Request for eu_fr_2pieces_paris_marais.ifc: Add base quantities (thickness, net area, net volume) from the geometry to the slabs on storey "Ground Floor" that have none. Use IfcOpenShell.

First a look at what the model holds.

```python
import ifcopenshell
import ifcopenshell.util.element
import ifcopenshell.util.unit

model = ifcopenshell.open("eu_fr_2pieces_paris_marais.ifc")
print(model.schema)
for unit_type in ("LENGTHUNIT", "AREAUNIT", "VOLUMEUNIT"):
    print(unit_type, ifcopenshell.util.unit.calculate_unit_scale(model, unit_type))
storey = next(s for s in model.by_type("IfcBuildingStorey") if s.Name == "Ground Floor")
slabs = [e for e in ifcopenshell.util.element.get_decomposition(storey) if e.is_a("IfcSlab")]
for e in sorted(slabs, key=lambda e: e.id()):
    print(e.id(), e.is_a(), e.Name, list(ifcopenshell.util.element.get_psets(e, qtos_only=True)), sep=" | ")
```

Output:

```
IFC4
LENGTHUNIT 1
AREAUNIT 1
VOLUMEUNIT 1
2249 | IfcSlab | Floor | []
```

```python
import ifcopenshell
import ifcopenshell.api.pset
import ifcopenshell.geom
import ifcopenshell.util.element
import ifcopenshell.util.shape
import ifcopenshell.util.unit

model = ifcopenshell.open("eu_fr_2pieces_paris_marais.ifc")
unit_scale = ifcopenshell.util.unit.calculate_unit_scale(model)
area_scale = ifcopenshell.util.unit.calculate_unit_scale(model, "AREAUNIT")
volume_scale = ifcopenshell.util.unit.calculate_unit_scale(model, "VOLUMEUNIT")
settings = ifcopenshell.geom.settings()

storey = next(s for s in model.by_type("IfcBuildingStorey") if s.Name == "Ground Floor")
slabs = [e for e in ifcopenshell.util.element.get_decomposition(storey) if e.is_a("IfcSlab")]

for e in sorted(slabs, key=lambda e: e.id()):
    if ifcopenshell.util.element.get_psets(e, qtos_only=True, should_inherit=False):
        continue
    # Geometry comes back in metres, in the element's own axes.
    shape = ifcopenshell.geom.create_shape(settings, e)
    values = {
        "Width": ifcopenshell.util.shape.get_z(shape.geometry) / unit_scale,
        "NetArea": ifcopenshell.util.shape.get_footprint_area(shape.geometry) / area_scale,
        "NetVolume": ifcopenshell.util.shape.get_volume(shape.geometry) / volume_scale,
    }
    qto = ifcopenshell.api.pset.add_qto(model, product=e, name="Qto_SlabBaseQuantities")
    ifcopenshell.api.pset.edit_qto(model, qto=qto, properties=values)
    print(e.id(), {k: round(v, 3) for k, v in values.items()})

model.write("eu_fr_2pieces_paris_marais_rev.ifc")
```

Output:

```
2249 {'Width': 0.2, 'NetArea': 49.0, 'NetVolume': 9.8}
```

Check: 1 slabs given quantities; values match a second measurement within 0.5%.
